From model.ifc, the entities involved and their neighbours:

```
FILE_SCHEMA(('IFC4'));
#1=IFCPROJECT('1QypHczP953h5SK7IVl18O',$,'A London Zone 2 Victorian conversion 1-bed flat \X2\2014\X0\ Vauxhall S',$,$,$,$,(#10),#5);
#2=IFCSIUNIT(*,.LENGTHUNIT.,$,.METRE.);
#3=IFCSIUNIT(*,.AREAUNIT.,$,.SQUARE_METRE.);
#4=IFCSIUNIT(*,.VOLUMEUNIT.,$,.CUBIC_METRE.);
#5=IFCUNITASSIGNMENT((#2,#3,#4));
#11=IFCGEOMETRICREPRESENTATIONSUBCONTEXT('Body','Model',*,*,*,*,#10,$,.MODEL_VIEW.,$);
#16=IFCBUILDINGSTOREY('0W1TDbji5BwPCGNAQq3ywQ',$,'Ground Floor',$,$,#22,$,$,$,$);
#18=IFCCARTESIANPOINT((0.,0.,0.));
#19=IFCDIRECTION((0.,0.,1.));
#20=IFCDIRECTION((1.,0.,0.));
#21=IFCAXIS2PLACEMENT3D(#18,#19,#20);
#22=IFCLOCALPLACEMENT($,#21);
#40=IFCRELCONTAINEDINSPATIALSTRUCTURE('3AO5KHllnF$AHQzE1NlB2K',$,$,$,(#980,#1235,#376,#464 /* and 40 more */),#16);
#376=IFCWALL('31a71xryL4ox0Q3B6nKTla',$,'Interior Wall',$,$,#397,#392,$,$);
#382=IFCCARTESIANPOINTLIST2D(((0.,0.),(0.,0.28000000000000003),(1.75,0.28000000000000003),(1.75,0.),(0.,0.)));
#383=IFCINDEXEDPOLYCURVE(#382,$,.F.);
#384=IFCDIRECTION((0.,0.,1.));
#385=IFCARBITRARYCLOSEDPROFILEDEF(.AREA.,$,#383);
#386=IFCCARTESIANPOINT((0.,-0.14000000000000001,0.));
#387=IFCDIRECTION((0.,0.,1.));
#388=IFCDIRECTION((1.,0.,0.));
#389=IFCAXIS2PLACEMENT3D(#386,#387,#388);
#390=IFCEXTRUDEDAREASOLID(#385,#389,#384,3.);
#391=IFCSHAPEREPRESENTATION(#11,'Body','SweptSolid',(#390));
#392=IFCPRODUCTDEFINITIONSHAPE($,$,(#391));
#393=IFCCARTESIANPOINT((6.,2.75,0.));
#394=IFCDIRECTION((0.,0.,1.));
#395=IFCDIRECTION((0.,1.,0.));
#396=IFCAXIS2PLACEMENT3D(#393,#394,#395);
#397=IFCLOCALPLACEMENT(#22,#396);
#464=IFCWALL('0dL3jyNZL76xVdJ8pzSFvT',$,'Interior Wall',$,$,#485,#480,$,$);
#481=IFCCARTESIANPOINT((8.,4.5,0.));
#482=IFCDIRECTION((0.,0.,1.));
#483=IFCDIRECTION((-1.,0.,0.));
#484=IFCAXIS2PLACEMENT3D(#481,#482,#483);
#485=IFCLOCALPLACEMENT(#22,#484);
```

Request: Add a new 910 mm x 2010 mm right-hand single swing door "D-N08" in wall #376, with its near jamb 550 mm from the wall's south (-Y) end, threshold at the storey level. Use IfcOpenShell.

```python
import numpy as np
import ifcopenshell
import ifcopenshell.api.feature
import ifcopenshell.api.geometry
import ifcopenshell.api.root
import ifcopenshell.api.spatial
import ifcopenshell.geom
import ifcopenshell.util.element
import ifcopenshell.util.placement
import ifcopenshell.util.representation
import ifcopenshell.util.shape
import ifcopenshell.util.unit

model = ifcopenshell.open("model.ifc")
unit_scale = ifcopenshell.util.unit.calculate_unit_scale(model)
settings = ifcopenshell.geom.settings()


def volume(element):
    """Net volume in cubic metres, openings subtracted."""
    shape = ifcopenshell.geom.create_shape(settings, element)
    return ifcopenshell.util.shape.get_volume(shape.geometry)


wall = model.by_id(376)
storey = ifcopenshell.util.element.get_container(wall, ifc_class="IfcBuildingStorey")
context = ifcopenshell.util.representation.get_context(model, "Model", "Body", "MODEL_VIEW")
before = volume(wall)

width, height, from_end, sill = 0.91, 2.01, 0.55, 0.0  # metres

# The wall runs along its own X axis, and the end named is its -X end.
wall_shape = ifcopenshell.geom.create_shape(settings, wall)
x, y, z = ifcopenshell.util.shape.get_vertices(wall_shape.geometry).T
start = x.min() + from_end
face, thickness = float(y.min()), float(y.max() - y.min())
wall_matrix = ifcopenshell.util.placement.get_local_placement(wall.ObjectPlacement)
level = ifcopenshell.util.placement.get_local_placement(storey.ObjectPlacement)[2, 3]


def in_wall(x, y):
    """Placement at x, y metres in the wall's axes, at sill height."""
    matrix = wall_matrix.copy()
    matrix[:, 3] = wall_matrix @ np.array([x / unit_scale, y / unit_scale, 0.0, 1.0])
    matrix[2, 3] = level + sill / unit_scale
    return matrix


# Opening: a box that overshoots both wall faces by 50 mm.
opening = ifcopenshell.api.root.create_entity(model, ifc_class="IfcOpeningElement", predefined_type="OPENING")
box = ifcopenshell.api.geometry.add_wall_representation(
    model, context=context, length=width, height=height, thickness=thickness + 0.1
)
ifcopenshell.api.geometry.assign_representation(model, product=opening, representation=box)
ifcopenshell.api.geometry.edit_object_placement(model, product=opening, matrix=in_wall(start, face - 0.05), is_si=False)
ifcopenshell.api.feature.add_feature(model, feature=opening, element=wall)

door = ifcopenshell.api.root.create_entity(model, ifc_class="IfcDoor", name="D-N08", predefined_type="DOOR")
door.OverallWidth, door.OverallHeight = width / unit_scale, height / unit_scale
door.OperationType = "SINGLE_SWING_RIGHT"
body = ifcopenshell.api.geometry.add_door_representation(
    model,
    context=context,
    overall_width=door.OverallWidth,
    overall_height=door.OverallHeight,
    operation_type="SINGLE_SWING_RIGHT",
    lining_properties={"LiningDepth": thickness / unit_scale, "ThresholdDepth": thickness / unit_scale},
)
ifcopenshell.api.geometry.assign_representation(model, product=door, representation=body)
ifcopenshell.api.spatial.assign_container(model, products=[door], relating_structure=storey)
ifcopenshell.api.feature.add_filling(model, opening=opening, element=door)

# The lining spans the wall, so the door starts at the wall face.
ifcopenshell.api.geometry.edit_object_placement(model, product=door, matrix=in_wall(start, face), is_si=False)

after = volume(wall)

print(f"wall volume {before:.3f} -> {after:.3f} m3")

model.write("model_rev.ifc")
```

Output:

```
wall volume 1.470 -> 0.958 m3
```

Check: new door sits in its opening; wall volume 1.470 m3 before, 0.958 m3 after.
